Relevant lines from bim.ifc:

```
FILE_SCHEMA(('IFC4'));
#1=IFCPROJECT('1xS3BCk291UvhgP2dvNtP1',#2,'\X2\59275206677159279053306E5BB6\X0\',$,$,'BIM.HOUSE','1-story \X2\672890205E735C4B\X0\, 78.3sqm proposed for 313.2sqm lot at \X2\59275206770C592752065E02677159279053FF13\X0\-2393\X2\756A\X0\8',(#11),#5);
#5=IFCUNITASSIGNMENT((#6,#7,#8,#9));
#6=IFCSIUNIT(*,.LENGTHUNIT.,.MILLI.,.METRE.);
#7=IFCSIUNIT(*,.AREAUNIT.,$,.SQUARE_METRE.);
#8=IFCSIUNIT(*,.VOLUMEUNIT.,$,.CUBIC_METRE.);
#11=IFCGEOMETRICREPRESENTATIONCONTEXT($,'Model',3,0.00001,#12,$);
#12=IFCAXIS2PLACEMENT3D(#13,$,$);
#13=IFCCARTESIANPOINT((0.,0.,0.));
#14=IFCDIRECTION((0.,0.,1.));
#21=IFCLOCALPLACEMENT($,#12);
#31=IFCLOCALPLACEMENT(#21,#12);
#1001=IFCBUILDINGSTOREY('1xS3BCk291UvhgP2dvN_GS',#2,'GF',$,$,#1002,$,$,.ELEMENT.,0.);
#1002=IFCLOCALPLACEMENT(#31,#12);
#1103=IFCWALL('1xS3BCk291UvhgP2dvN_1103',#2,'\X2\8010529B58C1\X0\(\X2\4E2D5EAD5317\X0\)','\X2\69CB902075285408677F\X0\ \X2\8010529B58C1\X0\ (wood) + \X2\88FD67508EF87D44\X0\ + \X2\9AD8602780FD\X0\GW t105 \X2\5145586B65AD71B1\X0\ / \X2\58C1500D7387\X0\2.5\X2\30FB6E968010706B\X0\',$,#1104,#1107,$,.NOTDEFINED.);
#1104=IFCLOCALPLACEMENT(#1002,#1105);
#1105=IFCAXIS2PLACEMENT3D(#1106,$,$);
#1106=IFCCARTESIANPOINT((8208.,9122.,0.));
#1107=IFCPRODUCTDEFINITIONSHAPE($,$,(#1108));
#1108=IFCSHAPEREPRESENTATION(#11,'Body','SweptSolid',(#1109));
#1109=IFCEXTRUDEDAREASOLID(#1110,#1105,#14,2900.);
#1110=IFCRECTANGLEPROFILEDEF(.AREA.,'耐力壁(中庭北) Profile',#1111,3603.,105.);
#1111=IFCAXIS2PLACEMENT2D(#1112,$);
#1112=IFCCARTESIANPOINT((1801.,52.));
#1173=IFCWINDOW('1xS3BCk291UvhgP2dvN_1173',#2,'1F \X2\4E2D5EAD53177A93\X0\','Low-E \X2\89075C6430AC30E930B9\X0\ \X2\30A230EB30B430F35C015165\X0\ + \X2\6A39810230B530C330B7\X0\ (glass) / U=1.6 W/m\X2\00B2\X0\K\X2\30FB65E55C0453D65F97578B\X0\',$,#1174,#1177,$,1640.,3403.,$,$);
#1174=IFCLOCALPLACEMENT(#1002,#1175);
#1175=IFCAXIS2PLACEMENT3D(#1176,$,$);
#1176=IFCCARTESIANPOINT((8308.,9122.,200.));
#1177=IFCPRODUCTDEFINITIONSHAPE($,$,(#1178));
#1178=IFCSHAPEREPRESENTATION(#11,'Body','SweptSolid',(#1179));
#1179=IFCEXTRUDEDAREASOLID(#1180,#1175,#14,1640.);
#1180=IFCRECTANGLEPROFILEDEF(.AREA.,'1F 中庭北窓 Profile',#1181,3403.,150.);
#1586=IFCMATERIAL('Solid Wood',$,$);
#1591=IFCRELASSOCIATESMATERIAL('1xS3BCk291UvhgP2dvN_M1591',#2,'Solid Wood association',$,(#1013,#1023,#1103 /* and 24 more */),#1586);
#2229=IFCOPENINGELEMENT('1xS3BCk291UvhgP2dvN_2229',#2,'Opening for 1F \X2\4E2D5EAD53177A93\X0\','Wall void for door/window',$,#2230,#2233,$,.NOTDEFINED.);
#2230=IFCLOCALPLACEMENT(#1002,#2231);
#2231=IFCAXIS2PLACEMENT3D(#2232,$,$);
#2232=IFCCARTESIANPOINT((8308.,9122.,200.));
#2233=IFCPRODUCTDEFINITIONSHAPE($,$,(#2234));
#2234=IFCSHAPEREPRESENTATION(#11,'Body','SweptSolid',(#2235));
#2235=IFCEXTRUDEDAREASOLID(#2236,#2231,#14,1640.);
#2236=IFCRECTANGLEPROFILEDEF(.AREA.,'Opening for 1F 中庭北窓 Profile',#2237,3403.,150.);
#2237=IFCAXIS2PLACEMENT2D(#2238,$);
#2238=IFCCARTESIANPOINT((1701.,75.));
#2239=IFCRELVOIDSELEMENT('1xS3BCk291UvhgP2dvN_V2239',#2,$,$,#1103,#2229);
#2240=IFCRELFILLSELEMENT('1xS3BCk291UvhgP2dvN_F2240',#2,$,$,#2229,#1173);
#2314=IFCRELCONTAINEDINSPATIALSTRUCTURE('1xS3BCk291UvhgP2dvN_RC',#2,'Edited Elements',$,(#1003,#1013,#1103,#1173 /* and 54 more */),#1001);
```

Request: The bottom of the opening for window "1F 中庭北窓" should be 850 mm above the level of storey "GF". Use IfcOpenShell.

```python
import numpy as np
import ifcopenshell
import ifcopenshell.api.geometry
import ifcopenshell.geom
import ifcopenshell.util.element
import ifcopenshell.util.placement
import ifcopenshell.util.shape
import ifcopenshell.util.unit

model = ifcopenshell.open("bim.ifc")
unit_scale = ifcopenshell.util.unit.calculate_unit_scale(model)

window = model.by_id(1173)
opening = window.FillsVoids[0].RelatingOpeningElement
storey = ifcopenshell.util.element.get_container(window, ifc_class="IfcBuildingStorey")
level = ifcopenshell.util.placement.get_local_placement(storey.ObjectPlacement)[2, 3]

# The opening's origin need not be at the sill, so measure its lowest point.
shape = ifcopenshell.geom.create_shape(ifcopenshell.geom.settings(), opening)
bottom = ifcopenshell.util.shape.get_shape_bottom_elevation(shape, shape.geometry) / unit_scale
dz = level + 0.85 / unit_scale - bottom

shift = np.array([0.0, 0.0, dz])
# The window is not placed relative to its opening, so move both.
for product in (opening, window):
    matrix = ifcopenshell.util.placement.get_local_placement(product.ObjectPlacement)
    matrix[:3, 3] += shift
    ifcopenshell.api.geometry.edit_object_placement(model, product=product, matrix=matrix, is_si=False)

print(f"moved by {dz * unit_scale:+.3f} m")

model.write("bim_rev.ifc")
```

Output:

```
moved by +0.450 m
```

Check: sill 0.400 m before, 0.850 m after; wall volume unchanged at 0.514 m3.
